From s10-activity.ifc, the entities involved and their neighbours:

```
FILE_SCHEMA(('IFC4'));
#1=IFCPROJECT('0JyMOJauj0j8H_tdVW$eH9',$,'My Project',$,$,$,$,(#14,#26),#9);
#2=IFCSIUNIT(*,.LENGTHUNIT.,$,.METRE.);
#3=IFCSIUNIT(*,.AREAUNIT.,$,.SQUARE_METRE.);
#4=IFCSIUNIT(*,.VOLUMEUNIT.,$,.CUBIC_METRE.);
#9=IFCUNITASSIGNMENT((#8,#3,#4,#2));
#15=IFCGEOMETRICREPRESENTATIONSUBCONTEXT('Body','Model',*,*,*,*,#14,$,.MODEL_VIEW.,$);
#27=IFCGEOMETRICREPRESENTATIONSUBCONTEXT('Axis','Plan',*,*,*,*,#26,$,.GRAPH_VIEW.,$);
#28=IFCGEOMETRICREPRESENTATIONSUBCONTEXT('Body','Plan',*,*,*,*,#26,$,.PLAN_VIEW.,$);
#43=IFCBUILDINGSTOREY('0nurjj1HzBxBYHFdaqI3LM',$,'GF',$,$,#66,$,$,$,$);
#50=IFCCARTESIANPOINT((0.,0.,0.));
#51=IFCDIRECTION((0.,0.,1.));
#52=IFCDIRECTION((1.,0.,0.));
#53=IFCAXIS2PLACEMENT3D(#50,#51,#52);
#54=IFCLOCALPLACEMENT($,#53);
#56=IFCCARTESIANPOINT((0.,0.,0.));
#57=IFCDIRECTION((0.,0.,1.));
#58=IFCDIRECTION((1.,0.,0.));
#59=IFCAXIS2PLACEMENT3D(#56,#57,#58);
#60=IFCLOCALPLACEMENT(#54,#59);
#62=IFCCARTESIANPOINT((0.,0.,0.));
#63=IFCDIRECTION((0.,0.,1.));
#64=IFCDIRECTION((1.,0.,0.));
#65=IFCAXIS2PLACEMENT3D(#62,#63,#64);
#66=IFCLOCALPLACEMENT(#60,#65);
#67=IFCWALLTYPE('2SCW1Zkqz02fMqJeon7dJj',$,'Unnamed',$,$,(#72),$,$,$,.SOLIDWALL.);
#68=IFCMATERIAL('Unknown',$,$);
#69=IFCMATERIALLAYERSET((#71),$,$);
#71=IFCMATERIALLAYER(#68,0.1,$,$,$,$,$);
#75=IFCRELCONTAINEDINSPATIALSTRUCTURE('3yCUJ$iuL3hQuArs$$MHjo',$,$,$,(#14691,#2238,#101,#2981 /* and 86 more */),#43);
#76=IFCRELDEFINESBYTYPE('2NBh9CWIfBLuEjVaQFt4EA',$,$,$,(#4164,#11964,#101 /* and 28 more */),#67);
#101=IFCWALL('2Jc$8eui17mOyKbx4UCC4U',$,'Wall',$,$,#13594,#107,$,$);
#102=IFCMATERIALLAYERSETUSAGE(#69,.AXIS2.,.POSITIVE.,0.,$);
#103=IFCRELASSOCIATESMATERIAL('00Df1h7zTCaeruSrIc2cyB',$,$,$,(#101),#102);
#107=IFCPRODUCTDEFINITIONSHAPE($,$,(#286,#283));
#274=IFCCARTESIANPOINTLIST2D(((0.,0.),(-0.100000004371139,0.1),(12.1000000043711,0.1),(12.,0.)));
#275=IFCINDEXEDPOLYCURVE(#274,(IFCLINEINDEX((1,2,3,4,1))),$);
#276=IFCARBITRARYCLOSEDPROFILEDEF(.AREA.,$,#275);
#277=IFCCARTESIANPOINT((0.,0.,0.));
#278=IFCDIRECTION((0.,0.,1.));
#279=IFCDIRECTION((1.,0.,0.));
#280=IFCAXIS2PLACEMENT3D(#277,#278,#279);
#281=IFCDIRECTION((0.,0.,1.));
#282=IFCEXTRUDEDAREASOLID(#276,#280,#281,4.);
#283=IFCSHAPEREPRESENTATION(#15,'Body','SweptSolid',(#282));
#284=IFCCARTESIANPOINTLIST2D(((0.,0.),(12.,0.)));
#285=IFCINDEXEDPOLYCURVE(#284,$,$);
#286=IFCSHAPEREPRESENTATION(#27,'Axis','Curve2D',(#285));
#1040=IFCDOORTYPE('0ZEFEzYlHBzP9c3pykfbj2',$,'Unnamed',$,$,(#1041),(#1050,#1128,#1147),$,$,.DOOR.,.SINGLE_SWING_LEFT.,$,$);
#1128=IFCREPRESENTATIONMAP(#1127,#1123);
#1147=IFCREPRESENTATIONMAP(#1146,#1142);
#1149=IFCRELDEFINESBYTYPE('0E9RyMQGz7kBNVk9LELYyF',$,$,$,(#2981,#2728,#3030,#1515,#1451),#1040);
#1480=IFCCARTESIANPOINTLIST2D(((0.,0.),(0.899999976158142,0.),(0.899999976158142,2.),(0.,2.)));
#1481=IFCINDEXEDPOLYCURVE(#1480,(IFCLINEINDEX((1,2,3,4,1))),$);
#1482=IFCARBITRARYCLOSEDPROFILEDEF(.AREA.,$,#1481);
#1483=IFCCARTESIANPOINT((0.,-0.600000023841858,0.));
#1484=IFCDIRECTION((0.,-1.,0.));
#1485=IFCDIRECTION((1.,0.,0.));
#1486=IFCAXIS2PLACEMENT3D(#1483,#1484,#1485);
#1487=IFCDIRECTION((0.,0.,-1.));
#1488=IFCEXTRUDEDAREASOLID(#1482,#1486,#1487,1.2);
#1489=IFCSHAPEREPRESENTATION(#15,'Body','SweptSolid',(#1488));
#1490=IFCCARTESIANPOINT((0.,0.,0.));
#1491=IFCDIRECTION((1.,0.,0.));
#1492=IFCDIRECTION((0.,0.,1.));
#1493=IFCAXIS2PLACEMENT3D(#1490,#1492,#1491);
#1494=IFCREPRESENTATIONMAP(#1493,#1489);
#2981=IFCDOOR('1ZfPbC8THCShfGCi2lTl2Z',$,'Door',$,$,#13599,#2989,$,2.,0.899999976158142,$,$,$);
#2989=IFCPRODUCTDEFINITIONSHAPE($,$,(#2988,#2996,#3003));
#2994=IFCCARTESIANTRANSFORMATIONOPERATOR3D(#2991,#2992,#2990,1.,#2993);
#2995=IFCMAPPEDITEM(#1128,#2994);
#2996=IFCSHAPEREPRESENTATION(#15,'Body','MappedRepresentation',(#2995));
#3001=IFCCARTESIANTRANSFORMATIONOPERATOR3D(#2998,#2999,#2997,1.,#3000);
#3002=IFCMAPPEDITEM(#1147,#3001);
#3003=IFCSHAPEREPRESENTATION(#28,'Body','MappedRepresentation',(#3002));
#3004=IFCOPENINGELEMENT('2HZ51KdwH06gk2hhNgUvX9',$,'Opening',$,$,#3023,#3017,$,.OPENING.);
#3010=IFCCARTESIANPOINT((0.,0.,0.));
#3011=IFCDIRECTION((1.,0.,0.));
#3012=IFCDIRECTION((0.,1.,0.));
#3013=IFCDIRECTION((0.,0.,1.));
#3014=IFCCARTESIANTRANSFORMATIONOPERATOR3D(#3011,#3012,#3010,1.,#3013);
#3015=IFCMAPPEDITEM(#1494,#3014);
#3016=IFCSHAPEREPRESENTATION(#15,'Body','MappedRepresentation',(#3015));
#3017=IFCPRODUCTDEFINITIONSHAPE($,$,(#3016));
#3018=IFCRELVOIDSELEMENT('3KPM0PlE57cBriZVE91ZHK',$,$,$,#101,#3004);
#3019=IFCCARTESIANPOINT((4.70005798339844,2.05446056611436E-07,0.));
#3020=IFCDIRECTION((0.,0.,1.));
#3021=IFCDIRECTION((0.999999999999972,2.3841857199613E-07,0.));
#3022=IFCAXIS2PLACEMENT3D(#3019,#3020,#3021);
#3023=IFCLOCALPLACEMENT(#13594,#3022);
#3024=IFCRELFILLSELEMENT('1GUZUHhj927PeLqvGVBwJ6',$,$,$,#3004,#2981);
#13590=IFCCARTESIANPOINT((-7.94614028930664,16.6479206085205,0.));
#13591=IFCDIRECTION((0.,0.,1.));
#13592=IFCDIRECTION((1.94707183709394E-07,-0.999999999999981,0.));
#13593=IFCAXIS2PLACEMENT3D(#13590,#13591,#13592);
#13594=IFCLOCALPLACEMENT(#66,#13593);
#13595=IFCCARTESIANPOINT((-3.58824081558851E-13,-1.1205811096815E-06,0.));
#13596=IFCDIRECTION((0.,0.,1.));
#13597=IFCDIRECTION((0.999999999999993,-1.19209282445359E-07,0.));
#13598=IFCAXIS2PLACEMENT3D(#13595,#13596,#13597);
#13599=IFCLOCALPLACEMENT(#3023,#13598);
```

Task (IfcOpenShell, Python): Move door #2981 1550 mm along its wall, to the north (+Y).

```python
import ifcopenshell
import ifcopenshell.api.geometry
import ifcopenshell.util.placement
import ifcopenshell.util.unit

model = ifcopenshell.open("s10-activity.ifc")
unit_scale = ifcopenshell.util.unit.calculate_unit_scale(model)

door = model.by_guid("1ZfPbC8THCShfGCi2lTl2Z")
opening = door.FillsVoids[0].RelatingOpeningElement
wall = opening.VoidsElements[0].RelatingBuildingElement

wall_matrix = ifcopenshell.util.placement.get_local_placement(wall.ObjectPlacement)
shift = wall_matrix[:3, 0] * -1.55 / unit_scale
before = ifcopenshell.util.placement.get_local_placement(door.ObjectPlacement)[:3, 3].copy()

# The door is placed relative to its opening, so it follows when the opening moves.
matrix = ifcopenshell.util.placement.get_local_placement(opening.ObjectPlacement)
matrix[:3, 3] += shift
ifcopenshell.api.geometry.edit_object_placement(
    model, product=opening, matrix=matrix, is_si=False, should_transform_children=True
)

after = ifcopenshell.util.placement.get_local_placement(door.ObjectPlacement)[:3, 3]
print("door moved by", (after - before).round(3) + 0.0)

model.write("s10-activity_updated.ifc")
```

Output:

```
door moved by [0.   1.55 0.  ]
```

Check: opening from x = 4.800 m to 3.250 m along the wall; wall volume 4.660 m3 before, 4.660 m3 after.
